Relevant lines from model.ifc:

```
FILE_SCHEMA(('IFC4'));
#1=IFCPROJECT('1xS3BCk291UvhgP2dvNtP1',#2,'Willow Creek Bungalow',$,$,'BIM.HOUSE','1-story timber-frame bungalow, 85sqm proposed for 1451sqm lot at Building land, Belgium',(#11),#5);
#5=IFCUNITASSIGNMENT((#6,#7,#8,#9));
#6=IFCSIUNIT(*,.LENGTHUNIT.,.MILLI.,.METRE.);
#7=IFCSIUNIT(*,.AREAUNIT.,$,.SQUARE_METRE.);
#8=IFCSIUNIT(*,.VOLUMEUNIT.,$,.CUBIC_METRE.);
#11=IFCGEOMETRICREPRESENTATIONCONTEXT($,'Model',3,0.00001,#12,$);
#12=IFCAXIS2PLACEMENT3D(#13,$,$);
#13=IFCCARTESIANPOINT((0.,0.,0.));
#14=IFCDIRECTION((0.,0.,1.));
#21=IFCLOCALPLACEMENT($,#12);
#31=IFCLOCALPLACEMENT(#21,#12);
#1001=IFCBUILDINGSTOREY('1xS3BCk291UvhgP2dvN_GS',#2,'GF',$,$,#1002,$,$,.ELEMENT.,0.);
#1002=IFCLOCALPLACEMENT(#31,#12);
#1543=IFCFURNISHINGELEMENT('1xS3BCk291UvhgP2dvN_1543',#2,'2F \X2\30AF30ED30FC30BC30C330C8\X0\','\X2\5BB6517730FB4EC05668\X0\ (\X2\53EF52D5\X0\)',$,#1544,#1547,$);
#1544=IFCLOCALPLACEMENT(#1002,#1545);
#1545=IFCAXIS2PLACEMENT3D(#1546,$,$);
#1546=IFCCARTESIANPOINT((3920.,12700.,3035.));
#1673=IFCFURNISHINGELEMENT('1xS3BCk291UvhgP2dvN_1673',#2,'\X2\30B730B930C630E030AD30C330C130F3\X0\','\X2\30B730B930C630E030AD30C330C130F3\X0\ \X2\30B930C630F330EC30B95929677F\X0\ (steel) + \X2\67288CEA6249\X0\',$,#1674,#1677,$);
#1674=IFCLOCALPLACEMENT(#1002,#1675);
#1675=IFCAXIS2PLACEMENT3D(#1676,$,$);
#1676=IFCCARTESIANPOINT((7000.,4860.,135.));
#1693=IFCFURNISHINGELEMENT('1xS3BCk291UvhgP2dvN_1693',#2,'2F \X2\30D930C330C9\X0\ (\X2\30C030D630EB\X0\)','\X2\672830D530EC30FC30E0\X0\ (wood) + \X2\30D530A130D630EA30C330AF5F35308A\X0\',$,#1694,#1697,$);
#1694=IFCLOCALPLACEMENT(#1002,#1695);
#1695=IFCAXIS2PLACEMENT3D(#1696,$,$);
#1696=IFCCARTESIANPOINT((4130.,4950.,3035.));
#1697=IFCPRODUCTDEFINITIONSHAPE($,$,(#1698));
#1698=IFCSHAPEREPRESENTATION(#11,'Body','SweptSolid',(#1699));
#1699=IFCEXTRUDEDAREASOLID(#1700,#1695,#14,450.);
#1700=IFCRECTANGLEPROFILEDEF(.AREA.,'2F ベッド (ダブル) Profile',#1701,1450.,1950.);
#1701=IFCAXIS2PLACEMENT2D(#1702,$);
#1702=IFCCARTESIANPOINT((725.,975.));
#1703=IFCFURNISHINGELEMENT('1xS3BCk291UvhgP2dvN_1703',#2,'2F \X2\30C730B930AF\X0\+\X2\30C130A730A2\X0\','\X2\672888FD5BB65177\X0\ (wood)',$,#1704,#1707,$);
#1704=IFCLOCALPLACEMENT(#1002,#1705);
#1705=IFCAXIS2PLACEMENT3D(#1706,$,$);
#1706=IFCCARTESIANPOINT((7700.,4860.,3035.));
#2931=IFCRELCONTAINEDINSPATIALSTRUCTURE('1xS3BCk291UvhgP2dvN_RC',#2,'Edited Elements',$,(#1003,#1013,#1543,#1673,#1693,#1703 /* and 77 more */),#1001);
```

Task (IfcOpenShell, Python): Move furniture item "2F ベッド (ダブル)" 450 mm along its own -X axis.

```python
import ifcopenshell
import ifcopenshell.api.geometry
import ifcopenshell.util.placement

model = ifcopenshell.open("model.ifc")

item = model.by_guid("1xS3BCk291UvhgP2dvN_1693")
matrix = ifcopenshell.util.placement.get_local_placement(item.ObjectPlacement)
matrix[:3, 3] -= matrix[:3, 0] * 450.0
ifcopenshell.api.geometry.edit_object_placement(model, product=item, matrix=matrix, is_si=False)

print(ifcopenshell.util.placement.get_local_placement(item.ObjectPlacement).round(3) + 0.0)

model.write("model_edited.ifc")
```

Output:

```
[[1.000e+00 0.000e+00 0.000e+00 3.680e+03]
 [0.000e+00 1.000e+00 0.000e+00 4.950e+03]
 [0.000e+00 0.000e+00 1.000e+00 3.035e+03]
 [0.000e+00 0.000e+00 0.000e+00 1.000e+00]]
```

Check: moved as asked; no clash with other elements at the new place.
